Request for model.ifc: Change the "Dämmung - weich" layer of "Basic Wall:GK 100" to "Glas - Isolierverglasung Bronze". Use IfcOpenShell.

First a look at what the model holds.

```python
import ifcopenshell
import ifcopenshell.util.element

model = ifcopenshell.open("model.ifc")
print(model.schema)
for layer_set in model.by_type("IfcMaterialLayerSet"):
    if layer_set.LayerSetName == "Basic Wall:GK 100":
        for layer in layer_set.MaterialLayers:
            print(layer.id(), layer.Material and layer.Material.Name, layer.LayerThickness, sep=" | ")
        print(len(ifcopenshell.util.element.get_elements_by_material(model, layer_set)), "elements and types use it")
print(sorted(m.Name for m in model.by_type("IfcMaterial") if m.Name)[:60])
```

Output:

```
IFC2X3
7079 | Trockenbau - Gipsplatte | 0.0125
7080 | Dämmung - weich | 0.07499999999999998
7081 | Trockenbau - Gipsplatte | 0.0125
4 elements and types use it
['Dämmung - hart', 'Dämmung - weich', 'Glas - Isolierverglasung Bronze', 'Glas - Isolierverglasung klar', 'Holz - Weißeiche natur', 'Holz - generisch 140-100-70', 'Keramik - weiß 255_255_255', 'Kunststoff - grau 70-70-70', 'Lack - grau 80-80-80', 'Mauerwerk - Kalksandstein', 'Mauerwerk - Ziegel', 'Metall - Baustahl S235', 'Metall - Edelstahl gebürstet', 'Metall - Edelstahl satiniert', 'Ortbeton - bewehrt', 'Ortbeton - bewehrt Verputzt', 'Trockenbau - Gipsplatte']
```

```python
import ifcopenshell
import ifcopenshell.api.material

model = ifcopenshell.open("model.ifc")

layer_set = next(s for s in model.by_type("IfcMaterialLayerSet") if s.LayerSetName == "Basic Wall:GK 100")
layer = next(l for l in layer_set.MaterialLayers if l.Material and l.Material.Name == "Dämmung - weich")
material = next(m for m in model.by_type("IfcMaterial") if m.Name == "Glas - Isolierverglasung Bronze")

# Point this one layer at the other material; renaming the old one would change it everywhere.
ifcopenshell.api.material.edit_layer(model, layer=layer, attributes={}, material=material)

print([l.Material.Name if l.Material else None for l in layer_set.MaterialLayers])

model.write("model_rev.ifc")
```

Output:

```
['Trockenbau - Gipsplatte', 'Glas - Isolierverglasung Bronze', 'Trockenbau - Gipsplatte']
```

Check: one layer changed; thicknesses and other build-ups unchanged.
